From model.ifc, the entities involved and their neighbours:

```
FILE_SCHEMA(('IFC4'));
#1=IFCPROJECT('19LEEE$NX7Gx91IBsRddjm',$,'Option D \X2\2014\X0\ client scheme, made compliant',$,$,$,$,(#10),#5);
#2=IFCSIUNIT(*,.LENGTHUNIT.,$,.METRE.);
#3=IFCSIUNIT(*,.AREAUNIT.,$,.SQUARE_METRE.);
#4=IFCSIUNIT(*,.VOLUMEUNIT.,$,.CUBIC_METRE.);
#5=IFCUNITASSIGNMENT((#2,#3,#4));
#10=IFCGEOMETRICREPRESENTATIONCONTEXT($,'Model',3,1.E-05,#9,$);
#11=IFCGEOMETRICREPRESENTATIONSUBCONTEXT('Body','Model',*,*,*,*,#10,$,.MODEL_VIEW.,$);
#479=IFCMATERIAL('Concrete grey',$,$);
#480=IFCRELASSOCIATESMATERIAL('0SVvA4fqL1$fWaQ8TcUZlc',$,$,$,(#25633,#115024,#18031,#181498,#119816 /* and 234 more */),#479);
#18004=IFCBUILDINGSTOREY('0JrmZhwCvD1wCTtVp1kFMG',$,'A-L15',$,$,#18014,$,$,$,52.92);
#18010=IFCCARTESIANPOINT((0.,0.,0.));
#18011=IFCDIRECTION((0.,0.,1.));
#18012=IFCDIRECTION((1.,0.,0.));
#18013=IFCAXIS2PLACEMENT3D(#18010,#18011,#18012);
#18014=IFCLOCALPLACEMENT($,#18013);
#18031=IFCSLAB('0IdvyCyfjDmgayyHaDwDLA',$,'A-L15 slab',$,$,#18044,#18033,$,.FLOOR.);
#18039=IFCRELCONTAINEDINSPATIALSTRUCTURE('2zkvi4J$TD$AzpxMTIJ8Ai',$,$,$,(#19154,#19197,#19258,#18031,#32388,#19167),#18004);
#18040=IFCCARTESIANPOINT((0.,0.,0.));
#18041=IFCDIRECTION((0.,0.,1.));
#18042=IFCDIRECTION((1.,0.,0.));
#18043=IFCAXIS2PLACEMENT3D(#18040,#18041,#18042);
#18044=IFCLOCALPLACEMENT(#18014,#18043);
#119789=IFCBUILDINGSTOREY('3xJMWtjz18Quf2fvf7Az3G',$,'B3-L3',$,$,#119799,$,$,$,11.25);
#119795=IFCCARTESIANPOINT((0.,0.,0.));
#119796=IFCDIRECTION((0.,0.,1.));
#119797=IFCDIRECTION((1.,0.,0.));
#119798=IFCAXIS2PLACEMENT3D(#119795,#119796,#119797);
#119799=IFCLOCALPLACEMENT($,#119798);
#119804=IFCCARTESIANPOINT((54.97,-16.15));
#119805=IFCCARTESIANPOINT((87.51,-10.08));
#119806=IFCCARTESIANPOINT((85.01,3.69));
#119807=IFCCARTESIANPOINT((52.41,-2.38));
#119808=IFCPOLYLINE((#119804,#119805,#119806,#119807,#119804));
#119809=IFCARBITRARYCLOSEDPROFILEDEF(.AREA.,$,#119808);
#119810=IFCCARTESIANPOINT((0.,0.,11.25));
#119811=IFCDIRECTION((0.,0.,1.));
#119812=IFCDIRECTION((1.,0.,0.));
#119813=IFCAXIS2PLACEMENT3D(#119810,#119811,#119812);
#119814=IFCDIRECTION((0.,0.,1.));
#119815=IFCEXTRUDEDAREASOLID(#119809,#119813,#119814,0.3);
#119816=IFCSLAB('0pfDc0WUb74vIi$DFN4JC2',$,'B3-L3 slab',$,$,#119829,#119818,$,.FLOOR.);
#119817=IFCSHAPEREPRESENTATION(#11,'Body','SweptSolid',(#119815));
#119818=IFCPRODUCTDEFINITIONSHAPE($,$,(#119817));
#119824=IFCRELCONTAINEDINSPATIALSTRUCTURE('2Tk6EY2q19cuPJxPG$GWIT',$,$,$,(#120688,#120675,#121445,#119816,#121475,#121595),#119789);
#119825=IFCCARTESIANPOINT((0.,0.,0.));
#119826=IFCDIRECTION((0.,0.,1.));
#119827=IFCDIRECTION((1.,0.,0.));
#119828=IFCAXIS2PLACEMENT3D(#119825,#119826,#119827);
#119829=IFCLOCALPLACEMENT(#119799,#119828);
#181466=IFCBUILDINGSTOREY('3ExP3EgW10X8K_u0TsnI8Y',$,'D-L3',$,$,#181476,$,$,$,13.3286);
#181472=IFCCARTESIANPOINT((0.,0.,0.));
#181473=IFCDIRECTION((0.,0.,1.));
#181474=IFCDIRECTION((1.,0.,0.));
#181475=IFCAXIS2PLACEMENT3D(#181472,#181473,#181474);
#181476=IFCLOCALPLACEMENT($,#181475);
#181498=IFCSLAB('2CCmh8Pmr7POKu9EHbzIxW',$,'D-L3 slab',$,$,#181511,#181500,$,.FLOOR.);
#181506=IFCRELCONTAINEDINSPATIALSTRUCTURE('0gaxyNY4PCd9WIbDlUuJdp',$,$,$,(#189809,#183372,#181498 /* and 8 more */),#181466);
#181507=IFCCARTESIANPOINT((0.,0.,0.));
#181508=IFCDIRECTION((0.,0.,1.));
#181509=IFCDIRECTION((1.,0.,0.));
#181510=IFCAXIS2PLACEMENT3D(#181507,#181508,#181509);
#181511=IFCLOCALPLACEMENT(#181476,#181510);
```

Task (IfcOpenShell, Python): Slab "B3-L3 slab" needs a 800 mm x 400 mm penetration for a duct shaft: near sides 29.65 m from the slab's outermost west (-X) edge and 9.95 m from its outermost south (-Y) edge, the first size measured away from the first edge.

```python
import numpy as np
import ifcopenshell
import ifcopenshell.api.feature
import ifcopenshell.api.geometry
import ifcopenshell.api.root
import ifcopenshell.geom
import ifcopenshell.util.placement
import ifcopenshell.util.representation
import ifcopenshell.util.shape
import ifcopenshell.util.unit

model = ifcopenshell.open("model.ifc")
unit_scale = ifcopenshell.util.unit.calculate_unit_scale(model)
settings = ifcopenshell.geom.settings()


def volume(element):
    """Net volume in cubic metres, openings subtracted."""
    shape = ifcopenshell.geom.create_shape(settings, element)
    return ifcopenshell.util.shape.get_volume(shape.geometry)


slab = model.by_id(119816)
before = volume(slab)

# Extent in the slab's own axes, in metres. The edges named are its -X and -Y sides.
slab_shape = ifcopenshell.geom.create_shape(settings, slab)
vertices = ifcopenshell.util.shape.get_vertices(slab_shape.geometry)
x_min, y_min, bottom = vertices.min(axis=0)
top = vertices[:, 2].max()

opening = ifcopenshell.api.root.create_entity(model, ifc_class="IfcOpeningElement", name="Duct shaft opening", predefined_type="OPENING")
context = ifcopenshell.util.representation.get_context(model, "Model", "Body", "MODEL_VIEW")
width, depth = 0.8, 0.4
outline = [(0.0, 0.0), (width, 0.0), (width, depth), (0.0, depth), (0.0, 0.0)]
# Overshoot both faces by 50 mm so the cut is clean.
shape = ifcopenshell.api.geometry.add_slab_representation(
    model, context=context, depth=top - bottom + 0.1, polyline=outline
)
ifcopenshell.api.geometry.assign_representation(model, product=opening, representation=shape)

matrix = ifcopenshell.util.placement.get_local_placement(slab.ObjectPlacement)
matrix[:, 3] = matrix @ np.append(np.array([x_min + 29.65, y_min + 9.95, bottom - 0.05]) / unit_scale, 1.0)
ifcopenshell.api.geometry.edit_object_placement(model, product=opening, matrix=matrix, is_si=False)
ifcopenshell.api.feature.add_feature(model, feature=opening, element=slab)

after = volume(slab)

print(f"slab volume {before:.3f} -> {after:.3f} m3")

model.write("model-out.ifc")
```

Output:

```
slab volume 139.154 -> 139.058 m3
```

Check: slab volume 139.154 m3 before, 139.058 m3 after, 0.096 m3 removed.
